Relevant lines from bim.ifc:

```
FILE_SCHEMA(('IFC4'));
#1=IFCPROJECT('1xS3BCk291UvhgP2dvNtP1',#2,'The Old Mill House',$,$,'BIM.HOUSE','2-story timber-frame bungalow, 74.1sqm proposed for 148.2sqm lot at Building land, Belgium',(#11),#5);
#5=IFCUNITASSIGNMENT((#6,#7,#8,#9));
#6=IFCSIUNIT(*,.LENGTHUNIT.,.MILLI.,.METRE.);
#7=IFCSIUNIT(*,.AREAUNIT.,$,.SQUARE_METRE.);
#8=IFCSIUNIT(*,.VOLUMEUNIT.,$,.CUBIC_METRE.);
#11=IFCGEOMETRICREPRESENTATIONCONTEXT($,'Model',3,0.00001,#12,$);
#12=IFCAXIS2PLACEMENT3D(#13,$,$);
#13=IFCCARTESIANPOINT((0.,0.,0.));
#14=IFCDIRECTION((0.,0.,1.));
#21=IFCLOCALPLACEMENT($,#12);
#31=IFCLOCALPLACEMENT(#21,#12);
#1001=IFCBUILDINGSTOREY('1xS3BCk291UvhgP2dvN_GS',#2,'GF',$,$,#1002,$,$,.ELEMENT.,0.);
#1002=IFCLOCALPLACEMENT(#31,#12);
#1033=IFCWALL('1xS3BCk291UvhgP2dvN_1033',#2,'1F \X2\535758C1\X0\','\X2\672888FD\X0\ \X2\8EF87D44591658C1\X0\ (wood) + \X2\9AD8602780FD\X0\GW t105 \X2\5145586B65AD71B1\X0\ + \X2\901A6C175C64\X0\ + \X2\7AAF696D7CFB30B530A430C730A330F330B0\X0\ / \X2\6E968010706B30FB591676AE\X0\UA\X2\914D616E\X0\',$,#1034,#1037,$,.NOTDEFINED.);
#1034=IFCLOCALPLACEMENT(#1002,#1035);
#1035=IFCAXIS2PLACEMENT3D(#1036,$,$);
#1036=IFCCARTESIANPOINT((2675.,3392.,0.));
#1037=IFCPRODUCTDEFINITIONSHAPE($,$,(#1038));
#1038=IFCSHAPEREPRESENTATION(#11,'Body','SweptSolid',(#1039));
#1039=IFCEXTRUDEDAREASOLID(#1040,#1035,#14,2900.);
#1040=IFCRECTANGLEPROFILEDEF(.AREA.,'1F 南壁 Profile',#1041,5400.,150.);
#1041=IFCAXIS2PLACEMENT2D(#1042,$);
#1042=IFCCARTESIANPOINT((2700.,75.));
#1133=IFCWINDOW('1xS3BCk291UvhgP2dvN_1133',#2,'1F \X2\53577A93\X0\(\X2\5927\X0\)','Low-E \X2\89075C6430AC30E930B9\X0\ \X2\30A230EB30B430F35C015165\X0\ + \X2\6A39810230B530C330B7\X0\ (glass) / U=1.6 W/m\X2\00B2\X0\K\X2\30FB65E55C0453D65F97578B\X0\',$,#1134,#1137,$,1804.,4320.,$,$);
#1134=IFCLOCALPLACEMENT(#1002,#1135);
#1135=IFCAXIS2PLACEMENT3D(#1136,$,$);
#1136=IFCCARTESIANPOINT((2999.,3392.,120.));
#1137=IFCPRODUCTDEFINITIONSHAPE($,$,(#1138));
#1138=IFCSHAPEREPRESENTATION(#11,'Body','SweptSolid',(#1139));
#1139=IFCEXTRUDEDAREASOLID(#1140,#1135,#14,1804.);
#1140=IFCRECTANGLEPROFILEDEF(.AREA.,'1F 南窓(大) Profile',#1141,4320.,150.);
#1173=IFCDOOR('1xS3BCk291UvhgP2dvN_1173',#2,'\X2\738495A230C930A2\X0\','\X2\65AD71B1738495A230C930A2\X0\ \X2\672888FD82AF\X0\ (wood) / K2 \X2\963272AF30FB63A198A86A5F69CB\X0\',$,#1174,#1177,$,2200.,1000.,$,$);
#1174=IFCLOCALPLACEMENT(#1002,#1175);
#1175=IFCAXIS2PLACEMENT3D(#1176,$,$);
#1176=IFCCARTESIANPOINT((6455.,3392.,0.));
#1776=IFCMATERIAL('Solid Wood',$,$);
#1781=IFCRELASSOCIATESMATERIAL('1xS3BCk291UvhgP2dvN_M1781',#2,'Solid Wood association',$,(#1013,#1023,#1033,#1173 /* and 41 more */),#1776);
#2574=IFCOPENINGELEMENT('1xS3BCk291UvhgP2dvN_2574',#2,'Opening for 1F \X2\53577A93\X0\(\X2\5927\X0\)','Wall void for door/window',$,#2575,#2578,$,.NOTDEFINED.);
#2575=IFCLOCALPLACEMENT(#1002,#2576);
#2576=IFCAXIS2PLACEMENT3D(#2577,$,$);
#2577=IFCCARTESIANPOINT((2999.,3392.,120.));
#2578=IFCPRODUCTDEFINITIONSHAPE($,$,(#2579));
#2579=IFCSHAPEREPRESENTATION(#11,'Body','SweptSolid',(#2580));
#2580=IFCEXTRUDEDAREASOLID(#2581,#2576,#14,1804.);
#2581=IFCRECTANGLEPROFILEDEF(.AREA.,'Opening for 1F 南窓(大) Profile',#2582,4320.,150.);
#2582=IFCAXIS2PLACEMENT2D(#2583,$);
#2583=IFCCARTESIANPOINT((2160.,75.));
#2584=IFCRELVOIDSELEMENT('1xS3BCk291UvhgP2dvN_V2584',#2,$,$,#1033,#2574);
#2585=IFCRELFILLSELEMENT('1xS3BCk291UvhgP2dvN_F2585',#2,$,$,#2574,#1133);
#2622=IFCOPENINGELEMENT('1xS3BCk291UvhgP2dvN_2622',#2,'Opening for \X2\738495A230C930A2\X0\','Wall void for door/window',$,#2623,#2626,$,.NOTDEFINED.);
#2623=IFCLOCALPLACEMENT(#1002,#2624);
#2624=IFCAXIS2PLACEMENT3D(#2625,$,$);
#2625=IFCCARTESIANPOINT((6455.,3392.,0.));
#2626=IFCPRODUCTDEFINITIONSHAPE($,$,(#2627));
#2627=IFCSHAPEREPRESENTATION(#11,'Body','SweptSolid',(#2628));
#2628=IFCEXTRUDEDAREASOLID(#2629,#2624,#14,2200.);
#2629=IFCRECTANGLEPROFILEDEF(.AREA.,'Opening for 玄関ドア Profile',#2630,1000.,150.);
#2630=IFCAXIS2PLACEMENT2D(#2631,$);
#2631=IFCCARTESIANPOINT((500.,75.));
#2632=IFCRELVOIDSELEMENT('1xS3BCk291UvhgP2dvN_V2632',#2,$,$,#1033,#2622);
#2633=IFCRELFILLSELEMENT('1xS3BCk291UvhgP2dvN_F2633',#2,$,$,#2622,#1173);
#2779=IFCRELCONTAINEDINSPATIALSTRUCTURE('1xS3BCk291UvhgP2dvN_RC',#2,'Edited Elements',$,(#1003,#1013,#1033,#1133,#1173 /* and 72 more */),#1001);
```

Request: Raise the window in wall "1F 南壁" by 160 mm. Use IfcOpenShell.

```python
import numpy as np
import ifcopenshell
import ifcopenshell.api.geometry
import ifcopenshell.util.placement
import ifcopenshell.util.unit

model = ifcopenshell.open("bim.ifc")
unit_scale = ifcopenshell.util.unit.calculate_unit_scale(model)

window = model.by_guid("1xS3BCk291UvhgP2dvN_1133")
opening = window.FillsVoids[0].RelatingOpeningElement
dz = 0.16 / unit_scale

shift = np.array([0.0, 0.0, dz])
# The window is not placed relative to its opening, so move both.
for product in (opening, window):
    matrix = ifcopenshell.util.placement.get_local_placement(product.ObjectPlacement)
    matrix[:3, 3] += shift
    ifcopenshell.api.geometry.edit_object_placement(model, product=product, matrix=matrix, is_si=False)

print(f"moved by {dz * unit_scale:+.3f} m")

model.write("bim_updated.ifc")
```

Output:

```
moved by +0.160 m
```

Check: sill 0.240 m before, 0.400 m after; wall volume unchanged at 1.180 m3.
